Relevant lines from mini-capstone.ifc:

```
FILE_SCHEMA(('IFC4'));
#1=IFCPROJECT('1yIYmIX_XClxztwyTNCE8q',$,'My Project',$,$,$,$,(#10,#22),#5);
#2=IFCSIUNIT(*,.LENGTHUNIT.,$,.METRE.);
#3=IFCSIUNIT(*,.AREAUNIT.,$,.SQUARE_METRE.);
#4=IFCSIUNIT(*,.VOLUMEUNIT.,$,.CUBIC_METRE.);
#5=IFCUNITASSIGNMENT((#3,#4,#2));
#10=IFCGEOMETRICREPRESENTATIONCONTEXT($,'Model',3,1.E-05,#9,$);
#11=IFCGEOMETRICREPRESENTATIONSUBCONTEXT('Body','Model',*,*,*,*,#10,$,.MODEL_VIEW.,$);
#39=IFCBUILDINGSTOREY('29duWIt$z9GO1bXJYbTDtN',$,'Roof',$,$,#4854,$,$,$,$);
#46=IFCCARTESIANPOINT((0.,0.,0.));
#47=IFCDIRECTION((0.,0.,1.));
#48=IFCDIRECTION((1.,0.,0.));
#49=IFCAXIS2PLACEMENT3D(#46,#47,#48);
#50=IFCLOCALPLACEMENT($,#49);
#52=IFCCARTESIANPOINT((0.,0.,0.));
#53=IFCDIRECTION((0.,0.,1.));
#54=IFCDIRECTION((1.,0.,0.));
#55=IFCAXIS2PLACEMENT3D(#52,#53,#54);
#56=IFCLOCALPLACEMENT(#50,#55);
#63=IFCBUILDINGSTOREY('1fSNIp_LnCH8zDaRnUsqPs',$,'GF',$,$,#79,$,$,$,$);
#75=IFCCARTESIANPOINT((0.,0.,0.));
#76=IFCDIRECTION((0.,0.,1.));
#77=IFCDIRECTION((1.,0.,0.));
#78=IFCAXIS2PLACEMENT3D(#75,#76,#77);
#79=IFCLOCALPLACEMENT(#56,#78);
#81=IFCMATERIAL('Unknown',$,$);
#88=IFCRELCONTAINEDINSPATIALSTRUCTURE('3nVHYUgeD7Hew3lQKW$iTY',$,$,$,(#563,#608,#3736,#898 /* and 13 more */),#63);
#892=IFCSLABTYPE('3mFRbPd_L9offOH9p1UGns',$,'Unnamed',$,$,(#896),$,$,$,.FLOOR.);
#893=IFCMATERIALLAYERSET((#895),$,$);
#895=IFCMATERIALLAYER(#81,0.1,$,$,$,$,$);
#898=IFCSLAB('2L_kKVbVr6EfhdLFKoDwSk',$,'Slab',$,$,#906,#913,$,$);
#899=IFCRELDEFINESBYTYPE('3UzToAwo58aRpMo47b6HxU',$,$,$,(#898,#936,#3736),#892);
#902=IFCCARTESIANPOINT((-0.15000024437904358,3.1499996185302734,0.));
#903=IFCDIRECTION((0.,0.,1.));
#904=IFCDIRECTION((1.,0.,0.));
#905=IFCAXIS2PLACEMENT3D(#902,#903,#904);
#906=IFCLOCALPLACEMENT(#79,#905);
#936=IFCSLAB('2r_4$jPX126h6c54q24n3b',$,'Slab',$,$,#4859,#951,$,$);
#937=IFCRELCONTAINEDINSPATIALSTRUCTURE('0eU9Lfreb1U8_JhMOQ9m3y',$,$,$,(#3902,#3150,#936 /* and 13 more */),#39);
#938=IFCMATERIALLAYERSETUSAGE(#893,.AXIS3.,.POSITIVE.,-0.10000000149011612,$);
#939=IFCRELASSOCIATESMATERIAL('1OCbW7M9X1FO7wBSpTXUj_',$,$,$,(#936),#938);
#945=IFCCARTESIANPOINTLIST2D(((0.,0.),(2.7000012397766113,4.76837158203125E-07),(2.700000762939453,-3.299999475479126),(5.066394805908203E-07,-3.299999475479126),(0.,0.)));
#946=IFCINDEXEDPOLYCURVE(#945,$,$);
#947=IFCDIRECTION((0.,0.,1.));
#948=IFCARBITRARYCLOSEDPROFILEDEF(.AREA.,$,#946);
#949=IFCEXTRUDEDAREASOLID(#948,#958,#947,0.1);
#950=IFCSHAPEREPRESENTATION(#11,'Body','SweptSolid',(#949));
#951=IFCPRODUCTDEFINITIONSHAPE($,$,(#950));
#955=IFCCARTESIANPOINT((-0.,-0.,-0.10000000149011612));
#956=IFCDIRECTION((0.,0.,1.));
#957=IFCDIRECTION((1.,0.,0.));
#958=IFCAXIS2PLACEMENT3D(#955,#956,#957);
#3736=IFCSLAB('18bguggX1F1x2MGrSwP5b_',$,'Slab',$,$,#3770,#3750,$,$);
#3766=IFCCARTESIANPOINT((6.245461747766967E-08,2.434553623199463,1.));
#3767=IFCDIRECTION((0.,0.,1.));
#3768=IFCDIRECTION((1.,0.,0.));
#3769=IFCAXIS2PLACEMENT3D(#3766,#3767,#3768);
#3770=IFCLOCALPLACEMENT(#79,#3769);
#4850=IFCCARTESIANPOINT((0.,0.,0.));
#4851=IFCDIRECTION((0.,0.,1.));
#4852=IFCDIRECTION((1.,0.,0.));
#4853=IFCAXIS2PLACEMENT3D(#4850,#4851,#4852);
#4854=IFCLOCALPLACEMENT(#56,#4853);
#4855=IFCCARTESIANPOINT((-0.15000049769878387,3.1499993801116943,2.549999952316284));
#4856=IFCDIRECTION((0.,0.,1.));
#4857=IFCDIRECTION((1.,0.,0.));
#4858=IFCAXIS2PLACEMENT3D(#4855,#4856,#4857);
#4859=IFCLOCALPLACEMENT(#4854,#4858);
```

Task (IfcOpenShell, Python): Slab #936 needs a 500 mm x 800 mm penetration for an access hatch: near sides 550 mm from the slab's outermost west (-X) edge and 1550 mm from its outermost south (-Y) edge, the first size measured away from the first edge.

```python
import numpy as np
import ifcopenshell
import ifcopenshell.api.feature
import ifcopenshell.api.geometry
import ifcopenshell.api.root
import ifcopenshell.geom
import ifcopenshell.util.placement
import ifcopenshell.util.representation
import ifcopenshell.util.shape
import ifcopenshell.util.unit

model = ifcopenshell.open("mini-capstone.ifc")
unit_scale = ifcopenshell.util.unit.calculate_unit_scale(model)
settings = ifcopenshell.geom.settings()


def volume(element):
    """Net volume in cubic metres, openings subtracted."""
    shape = ifcopenshell.geom.create_shape(settings, element)
    return ifcopenshell.util.shape.get_volume(shape.geometry)


slab = model.by_guid("2r_4$jPX126h6c54q24n3b")
before = volume(slab)

# Extent in the slab's own axes, in metres. The edges named are its -X and -Y sides.
slab_shape = ifcopenshell.geom.create_shape(settings, slab)
vertices = ifcopenshell.util.shape.get_vertices(slab_shape.geometry)
x_min, y_min, bottom = vertices.min(axis=0)
top = vertices[:, 2].max()

opening = ifcopenshell.api.root.create_entity(model, ifc_class="IfcOpeningElement", name="Access hatch opening", predefined_type="OPENING")
context = ifcopenshell.util.representation.get_context(model, "Model", "Body", "MODEL_VIEW")
width, depth = 0.5, 0.8
outline = [(0.0, 0.0), (width, 0.0), (width, depth), (0.0, depth), (0.0, 0.0)]
# Overshoot both faces by 50 mm so the cut is clean.
shape = ifcopenshell.api.geometry.add_slab_representation(
    model, context=context, depth=top - bottom + 0.1, polyline=outline
)
ifcopenshell.api.geometry.assign_representation(model, product=opening, representation=shape)

matrix = ifcopenshell.util.placement.get_local_placement(slab.ObjectPlacement)
matrix[:, 3] = matrix @ np.append(np.array([x_min + 0.55, y_min + 1.55, bottom - 0.05]) / unit_scale, 1.0)
ifcopenshell.api.geometry.edit_object_placement(model, product=opening, matrix=matrix, is_si=False)
ifcopenshell.api.feature.add_feature(model, feature=opening, element=slab)

after = volume(slab)

print(f"slab volume {before:.3f} -> {after:.3f} m3")

model.write("mini-capstone-out.ifc")
```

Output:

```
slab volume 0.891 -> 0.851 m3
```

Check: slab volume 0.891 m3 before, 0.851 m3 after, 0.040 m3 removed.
